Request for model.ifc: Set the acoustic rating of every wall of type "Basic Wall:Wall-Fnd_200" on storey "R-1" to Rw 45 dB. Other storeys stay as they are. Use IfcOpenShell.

First a look at what the model holds.

```python
import ifcopenshell
import ifcopenshell.util.element

model = ifcopenshell.open("model.ifc")
print(model.schema)
storey = next(s for s in model.by_type("IfcBuildingStorey") if s.Name == "R-1")
walls = [e for e in ifcopenshell.util.element.get_decomposition(storey) if e.is_a("IfcWall")]
seen = {}
for e in walls:
    element_type = ifcopenshell.util.element.get_type(e)
    key = (element_type.Name if element_type != e and element_type else None, ifcopenshell.util.element.get_pset(e, "Pset_WallCommon", "AcousticRating"))
    seen[key] = seen.get(key, 0) + 1
for (name, value), count in sorted(seen.items(), key=str):
    print(count, "x", name, "|", value)
```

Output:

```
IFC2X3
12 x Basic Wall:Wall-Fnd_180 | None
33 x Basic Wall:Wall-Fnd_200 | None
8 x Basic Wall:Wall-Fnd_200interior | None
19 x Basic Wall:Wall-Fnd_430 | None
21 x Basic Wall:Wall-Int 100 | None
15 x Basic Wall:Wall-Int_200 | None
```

```python
import ifcopenshell
import ifcopenshell.api.pset
import ifcopenshell.util.element

model = ifcopenshell.open("model.ifc")

storey = next(s for s in model.by_type("IfcBuildingStorey") if s.Name == "R-1")
walls = [e for e in ifcopenshell.util.element.get_decomposition(storey) if e.is_a("IfcWall")]

count = 0
for e in walls:
    element_type = ifcopenshell.util.element.get_type(e)
    if element_type in (None, e) or element_type.Name != "Basic Wall:Wall-Fnd_200":
        continue
    # add_pset returns the element's existing set when there is one.
    pset = ifcopenshell.api.pset.add_pset(model, product=e, name="Pset_WallCommon")
    ifcopenshell.api.pset.edit_pset(model, pset=pset, properties={"AcousticRating": "Rw 45 dB"})
    count += 1

print(count, "walls updated")

model.write("model_updated.ifc")
```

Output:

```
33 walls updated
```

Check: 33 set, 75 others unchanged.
